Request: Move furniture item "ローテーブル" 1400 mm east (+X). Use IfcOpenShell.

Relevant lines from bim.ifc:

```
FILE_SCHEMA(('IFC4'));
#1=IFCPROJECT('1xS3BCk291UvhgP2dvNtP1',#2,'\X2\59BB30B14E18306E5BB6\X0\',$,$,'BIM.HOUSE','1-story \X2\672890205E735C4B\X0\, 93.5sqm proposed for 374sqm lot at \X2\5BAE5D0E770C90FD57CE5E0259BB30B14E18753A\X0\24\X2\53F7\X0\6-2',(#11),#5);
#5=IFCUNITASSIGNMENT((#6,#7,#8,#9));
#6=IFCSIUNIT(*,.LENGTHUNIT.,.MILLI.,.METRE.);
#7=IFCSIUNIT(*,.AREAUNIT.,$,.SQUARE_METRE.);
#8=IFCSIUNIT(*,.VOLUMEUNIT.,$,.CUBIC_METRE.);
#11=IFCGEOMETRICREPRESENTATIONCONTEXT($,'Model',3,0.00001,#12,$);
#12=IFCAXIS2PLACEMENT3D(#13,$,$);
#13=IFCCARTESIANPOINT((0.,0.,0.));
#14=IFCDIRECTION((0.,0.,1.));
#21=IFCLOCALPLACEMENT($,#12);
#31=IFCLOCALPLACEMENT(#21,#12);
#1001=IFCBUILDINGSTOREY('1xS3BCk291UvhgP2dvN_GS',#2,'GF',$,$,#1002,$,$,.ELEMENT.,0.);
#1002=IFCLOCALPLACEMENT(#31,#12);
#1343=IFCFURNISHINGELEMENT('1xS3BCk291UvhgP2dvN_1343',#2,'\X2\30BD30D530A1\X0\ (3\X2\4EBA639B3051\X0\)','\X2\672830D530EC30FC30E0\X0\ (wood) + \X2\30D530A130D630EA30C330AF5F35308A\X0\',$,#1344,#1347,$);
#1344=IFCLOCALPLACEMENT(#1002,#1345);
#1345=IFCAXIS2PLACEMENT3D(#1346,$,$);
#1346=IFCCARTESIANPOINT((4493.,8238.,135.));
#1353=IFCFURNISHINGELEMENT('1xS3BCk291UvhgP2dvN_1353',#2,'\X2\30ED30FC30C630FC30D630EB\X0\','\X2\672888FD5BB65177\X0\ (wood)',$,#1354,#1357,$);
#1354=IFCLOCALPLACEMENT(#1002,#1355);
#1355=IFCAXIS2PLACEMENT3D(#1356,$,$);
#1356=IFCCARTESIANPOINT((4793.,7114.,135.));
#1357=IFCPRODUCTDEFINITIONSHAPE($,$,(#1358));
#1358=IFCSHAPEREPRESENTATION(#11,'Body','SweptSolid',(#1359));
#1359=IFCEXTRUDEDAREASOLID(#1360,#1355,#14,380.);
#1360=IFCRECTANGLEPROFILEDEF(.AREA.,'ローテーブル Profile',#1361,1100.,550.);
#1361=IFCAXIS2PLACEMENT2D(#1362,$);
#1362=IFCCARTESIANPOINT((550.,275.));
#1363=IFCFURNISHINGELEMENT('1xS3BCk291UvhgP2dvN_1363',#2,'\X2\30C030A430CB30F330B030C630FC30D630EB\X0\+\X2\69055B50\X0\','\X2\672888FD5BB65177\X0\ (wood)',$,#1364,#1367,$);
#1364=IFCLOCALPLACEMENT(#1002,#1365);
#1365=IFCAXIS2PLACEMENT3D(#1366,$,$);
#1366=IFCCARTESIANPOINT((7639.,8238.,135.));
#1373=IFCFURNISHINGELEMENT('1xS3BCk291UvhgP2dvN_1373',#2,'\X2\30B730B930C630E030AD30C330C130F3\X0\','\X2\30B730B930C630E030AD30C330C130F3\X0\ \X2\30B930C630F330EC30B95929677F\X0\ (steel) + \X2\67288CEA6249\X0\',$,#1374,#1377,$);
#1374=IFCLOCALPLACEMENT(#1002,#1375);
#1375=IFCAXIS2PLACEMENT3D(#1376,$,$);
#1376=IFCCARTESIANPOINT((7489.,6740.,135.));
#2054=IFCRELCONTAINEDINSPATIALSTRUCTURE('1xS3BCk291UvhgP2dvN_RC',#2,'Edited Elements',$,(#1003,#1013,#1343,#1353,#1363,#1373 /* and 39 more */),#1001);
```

```python
import ifcopenshell
import ifcopenshell.api.geometry
import ifcopenshell.util.placement
import ifcopenshell.util.unit

model = ifcopenshell.open("bim.ifc")
unit_scale = ifcopenshell.util.unit.calculate_unit_scale(model)

item = model.by_id(1353)
matrix = ifcopenshell.util.placement.get_local_placement(item.ObjectPlacement)
matrix[0, 3] += 1.4 / unit_scale
ifcopenshell.api.geometry.edit_object_placement(model, product=item, matrix=matrix, is_si=False)

print(ifcopenshell.util.placement.get_local_placement(item.ObjectPlacement).round(3) + 0.0)

model.write("bim_updated.ifc")
```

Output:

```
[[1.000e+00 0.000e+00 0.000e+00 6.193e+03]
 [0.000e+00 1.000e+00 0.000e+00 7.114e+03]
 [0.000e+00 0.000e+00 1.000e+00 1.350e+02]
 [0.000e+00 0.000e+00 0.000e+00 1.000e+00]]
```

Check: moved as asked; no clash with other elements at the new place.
